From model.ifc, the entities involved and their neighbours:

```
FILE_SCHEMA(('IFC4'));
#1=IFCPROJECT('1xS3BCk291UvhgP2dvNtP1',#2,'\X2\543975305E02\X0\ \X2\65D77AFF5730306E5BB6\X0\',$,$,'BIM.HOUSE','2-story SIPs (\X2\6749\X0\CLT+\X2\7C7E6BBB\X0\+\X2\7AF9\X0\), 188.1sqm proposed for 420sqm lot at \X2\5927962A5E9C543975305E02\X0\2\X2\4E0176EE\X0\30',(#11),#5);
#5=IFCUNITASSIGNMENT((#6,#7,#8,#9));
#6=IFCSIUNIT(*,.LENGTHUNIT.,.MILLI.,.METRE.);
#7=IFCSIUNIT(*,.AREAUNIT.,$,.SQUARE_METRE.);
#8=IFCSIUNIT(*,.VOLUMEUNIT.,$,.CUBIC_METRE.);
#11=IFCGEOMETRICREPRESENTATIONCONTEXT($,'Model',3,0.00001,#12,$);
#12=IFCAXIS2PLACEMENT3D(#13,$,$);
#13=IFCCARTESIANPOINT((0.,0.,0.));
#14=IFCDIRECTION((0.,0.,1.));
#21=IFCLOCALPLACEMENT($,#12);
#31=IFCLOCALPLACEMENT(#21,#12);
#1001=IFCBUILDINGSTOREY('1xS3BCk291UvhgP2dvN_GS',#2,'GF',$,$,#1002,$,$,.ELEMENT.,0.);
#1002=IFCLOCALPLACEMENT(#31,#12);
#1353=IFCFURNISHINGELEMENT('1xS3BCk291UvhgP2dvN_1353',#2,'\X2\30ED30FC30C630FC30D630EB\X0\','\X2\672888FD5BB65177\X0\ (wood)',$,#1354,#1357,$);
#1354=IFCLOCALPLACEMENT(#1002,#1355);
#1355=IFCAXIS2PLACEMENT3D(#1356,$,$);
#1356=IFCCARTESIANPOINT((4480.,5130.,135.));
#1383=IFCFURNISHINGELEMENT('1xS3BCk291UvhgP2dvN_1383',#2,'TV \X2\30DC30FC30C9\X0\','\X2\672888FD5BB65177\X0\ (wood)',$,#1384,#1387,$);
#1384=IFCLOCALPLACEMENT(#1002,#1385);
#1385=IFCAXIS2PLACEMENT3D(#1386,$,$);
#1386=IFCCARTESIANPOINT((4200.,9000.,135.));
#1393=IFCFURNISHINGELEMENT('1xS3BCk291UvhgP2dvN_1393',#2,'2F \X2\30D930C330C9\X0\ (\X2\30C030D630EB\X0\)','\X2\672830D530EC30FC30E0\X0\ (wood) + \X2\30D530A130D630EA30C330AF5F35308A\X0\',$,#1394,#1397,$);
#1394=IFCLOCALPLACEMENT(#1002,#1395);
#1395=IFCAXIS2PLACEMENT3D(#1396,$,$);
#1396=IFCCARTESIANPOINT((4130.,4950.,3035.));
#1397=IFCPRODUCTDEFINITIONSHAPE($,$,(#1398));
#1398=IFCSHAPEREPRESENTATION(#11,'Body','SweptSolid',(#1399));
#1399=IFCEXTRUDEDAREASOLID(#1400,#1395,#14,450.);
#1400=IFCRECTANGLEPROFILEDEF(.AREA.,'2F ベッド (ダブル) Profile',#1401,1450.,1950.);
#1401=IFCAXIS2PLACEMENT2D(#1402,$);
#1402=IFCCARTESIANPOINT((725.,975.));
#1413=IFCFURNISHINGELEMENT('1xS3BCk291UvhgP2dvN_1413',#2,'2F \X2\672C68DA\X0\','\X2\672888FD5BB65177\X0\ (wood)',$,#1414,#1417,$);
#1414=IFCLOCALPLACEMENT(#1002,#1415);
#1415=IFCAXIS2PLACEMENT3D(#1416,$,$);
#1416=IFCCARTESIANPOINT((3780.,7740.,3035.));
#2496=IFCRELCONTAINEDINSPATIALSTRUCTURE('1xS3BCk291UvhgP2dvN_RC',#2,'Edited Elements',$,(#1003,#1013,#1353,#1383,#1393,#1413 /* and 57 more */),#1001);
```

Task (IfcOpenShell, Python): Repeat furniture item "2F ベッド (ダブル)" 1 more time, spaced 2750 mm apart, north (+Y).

```python
import numpy as np
import ifcopenshell
import ifcopenshell.api.geometry
import ifcopenshell.api.root
import ifcopenshell.util.element
import ifcopenshell.util.placement
import ifcopenshell.util.unit

model = ifcopenshell.open("model.ifc")
unit_scale = ifcopenshell.util.unit.calculate_unit_scale(model)


def reuse_history(source, copy):
    """copy_class also copies each property set's owner history, people and application; keep the originals."""
    for rel in copy.IsDefinedBy:
        if rel.is_a("IfcRelDefinesByProperties") and (history := rel.RelatingPropertyDefinition.OwnerHistory):
            rel.RelatingPropertyDefinition.OwnerHistory = source.OwnerHistory
            ifcopenshell.util.element.remove_deep2(model, history)


source = model.by_guid("1xS3BCk291UvhgP2dvN_1393")
base = ifcopenshell.util.placement.get_local_placement(source.ObjectPlacement)
step = np.array([0.0, 1.0, 0.0]) * 2.75 / unit_scale

for i in range(1, 2):
    copy = ifcopenshell.api.root.copy_class(model, product=source)
    copy.Representation = ifcopenshell.util.element.copy_deep(
        model, source.Representation, exclude=["IfcGeometricRepresentationContext", "IfcRepresentationMap"]
    )
    reuse_history(source, copy)
    matrix = base.copy()
    matrix[:3, 3] += i * step
    print("added at", matrix[:3, 3].round(3) + 0.0)
    ifcopenshell.api.geometry.edit_object_placement(model, product=copy, matrix=matrix, is_si=False)

model.write("model_edited.ifc")
```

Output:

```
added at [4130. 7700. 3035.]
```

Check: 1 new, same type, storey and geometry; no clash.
